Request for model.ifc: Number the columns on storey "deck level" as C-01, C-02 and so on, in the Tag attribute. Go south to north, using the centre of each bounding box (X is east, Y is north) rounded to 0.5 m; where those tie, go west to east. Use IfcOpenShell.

First a look at what the model holds.

```python
import ifcopenshell
import ifcopenshell.util.element
import ifcopenshell.util.placement

model = ifcopenshell.open("model.ifc")
print(model.schema)
storey = next(s for s in model.by_type("IfcBuildingStorey") if s.Name == "deck level")
columns = [e for e in ifcopenshell.util.element.get_decomposition(storey) if e.is_a("IfcColumn")]
for e in sorted(columns, key=lambda e: e.id()):
    origin = ifcopenshell.util.placement.get_local_placement(e.ObjectPlacement)[:3, 3]
    print(e.id(), e.Tag, e.Name, origin.round(2) + 0.0, sep=" | ")
```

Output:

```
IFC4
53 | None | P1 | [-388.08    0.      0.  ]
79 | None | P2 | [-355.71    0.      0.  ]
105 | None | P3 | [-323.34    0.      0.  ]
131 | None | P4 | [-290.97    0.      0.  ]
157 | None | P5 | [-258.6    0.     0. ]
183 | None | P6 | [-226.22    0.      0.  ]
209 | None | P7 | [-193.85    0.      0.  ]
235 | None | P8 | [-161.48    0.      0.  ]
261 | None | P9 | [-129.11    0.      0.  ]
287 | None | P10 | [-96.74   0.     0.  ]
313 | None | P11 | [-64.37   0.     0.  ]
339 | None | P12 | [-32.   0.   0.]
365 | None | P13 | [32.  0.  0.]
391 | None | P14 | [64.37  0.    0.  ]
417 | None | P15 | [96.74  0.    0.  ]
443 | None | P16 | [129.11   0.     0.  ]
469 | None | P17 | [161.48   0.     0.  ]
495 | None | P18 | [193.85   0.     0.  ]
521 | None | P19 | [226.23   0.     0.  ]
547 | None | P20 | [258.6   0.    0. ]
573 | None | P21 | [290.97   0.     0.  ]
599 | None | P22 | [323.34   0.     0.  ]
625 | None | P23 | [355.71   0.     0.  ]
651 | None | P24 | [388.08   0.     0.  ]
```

```python
import ifcopenshell
import ifcopenshell.geom
import ifcopenshell.util.element
import ifcopenshell.util.shape

model = ifcopenshell.open("model.ifc")
settings = ifcopenshell.geom.settings()
settings.set("use-world-coords", True)


def centre(element):
    shape = ifcopenshell.geom.create_shape(settings, element)
    return ifcopenshell.util.shape.get_bbox_centroid(shape.geometry)


storey = next(s for s in model.by_type("IfcBuildingStorey") if s.Name == "deck level")
columns = [e for e in ifcopenshell.util.element.get_decomposition(storey) if e.is_a("IfcColumn")]

# Insertion points can sit at a corner or the storey origin, so sort by the geometry (in metres).
centres = {e: centre(e) for e in columns}
columns.sort(key=lambda e: (round(centres[e][1] / 0.5), centres[e][0]))

for i, e in enumerate(columns, start=1):
    number = f"C-{i:02d}"
    e.Tag = number
    print(e.id(), number)

model.write("model_v2.ifc")
```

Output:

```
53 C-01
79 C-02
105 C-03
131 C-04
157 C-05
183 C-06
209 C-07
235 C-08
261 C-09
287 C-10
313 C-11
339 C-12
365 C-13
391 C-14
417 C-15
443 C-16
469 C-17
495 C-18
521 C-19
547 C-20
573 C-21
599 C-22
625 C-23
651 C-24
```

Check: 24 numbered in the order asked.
